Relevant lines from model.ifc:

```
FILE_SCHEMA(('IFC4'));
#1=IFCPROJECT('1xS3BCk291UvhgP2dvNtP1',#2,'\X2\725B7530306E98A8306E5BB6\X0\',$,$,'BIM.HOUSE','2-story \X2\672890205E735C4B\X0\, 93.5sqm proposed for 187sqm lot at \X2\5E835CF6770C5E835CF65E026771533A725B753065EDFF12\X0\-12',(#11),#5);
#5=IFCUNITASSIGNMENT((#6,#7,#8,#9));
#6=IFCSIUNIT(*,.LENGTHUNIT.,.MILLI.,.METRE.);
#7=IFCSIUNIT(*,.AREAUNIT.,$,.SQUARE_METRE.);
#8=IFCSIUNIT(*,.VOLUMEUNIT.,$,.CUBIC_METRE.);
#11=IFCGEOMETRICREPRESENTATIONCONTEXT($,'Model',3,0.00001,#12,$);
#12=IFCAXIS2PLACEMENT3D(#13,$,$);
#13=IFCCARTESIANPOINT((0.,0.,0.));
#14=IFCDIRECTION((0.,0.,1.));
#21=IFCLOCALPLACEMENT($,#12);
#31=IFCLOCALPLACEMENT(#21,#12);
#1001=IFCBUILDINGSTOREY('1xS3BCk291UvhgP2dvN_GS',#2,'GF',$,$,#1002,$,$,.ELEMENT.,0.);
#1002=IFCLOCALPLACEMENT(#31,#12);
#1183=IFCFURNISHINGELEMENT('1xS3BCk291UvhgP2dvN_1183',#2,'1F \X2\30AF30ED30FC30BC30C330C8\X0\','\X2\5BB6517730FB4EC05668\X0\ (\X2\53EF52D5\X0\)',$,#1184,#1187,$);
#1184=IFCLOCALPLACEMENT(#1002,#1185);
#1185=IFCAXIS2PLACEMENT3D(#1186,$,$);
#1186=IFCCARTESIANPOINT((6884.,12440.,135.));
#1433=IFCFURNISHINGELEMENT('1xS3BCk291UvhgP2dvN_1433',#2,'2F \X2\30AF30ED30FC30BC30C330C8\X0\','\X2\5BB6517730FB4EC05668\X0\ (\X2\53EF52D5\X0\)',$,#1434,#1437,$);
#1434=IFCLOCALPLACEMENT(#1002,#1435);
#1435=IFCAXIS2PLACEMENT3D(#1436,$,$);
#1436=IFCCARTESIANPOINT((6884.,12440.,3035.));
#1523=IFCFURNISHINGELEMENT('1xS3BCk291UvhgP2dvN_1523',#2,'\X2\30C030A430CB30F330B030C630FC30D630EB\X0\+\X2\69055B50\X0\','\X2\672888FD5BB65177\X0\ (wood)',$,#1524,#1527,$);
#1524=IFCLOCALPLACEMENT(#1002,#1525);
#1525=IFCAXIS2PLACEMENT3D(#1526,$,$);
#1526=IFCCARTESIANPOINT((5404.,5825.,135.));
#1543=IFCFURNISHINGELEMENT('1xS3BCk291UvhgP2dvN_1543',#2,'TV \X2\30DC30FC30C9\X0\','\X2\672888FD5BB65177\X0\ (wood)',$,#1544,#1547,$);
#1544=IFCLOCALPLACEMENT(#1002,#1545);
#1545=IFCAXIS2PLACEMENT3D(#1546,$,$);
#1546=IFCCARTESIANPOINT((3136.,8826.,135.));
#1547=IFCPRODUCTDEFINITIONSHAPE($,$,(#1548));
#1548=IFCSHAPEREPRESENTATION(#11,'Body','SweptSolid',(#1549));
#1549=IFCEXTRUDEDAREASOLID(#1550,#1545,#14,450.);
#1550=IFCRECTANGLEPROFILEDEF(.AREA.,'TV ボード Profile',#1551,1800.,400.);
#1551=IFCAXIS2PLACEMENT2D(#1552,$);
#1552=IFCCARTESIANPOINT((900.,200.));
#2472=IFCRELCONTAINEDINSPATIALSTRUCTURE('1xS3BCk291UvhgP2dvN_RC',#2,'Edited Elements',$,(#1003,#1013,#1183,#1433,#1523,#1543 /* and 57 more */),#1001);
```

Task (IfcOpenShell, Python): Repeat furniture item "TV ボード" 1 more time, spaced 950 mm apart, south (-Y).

```python
import numpy as np
import ifcopenshell
import ifcopenshell.api.geometry
import ifcopenshell.api.root
import ifcopenshell.util.element
import ifcopenshell.util.placement
import ifcopenshell.util.unit

model = ifcopenshell.open("model.ifc")
unit_scale = ifcopenshell.util.unit.calculate_unit_scale(model)


def reuse_history(source, copy):
    """copy_class also copies each property set's owner history, people and application; keep the originals."""
    for rel in copy.IsDefinedBy:
        if rel.is_a("IfcRelDefinesByProperties") and (history := rel.RelatingPropertyDefinition.OwnerHistory):
            rel.RelatingPropertyDefinition.OwnerHistory = source.OwnerHistory
            ifcopenshell.util.element.remove_deep2(model, history)


source = model.by_id(1543)
base = ifcopenshell.util.placement.get_local_placement(source.ObjectPlacement)
step = np.array([0.0, -1.0, 0.0]) * 0.95 / unit_scale

for i in range(1, 2):
    copy = ifcopenshell.api.root.copy_class(model, product=source)
    copy.Representation = ifcopenshell.util.element.copy_deep(
        model, source.Representation, exclude=["IfcGeometricRepresentationContext", "IfcRepresentationMap"]
    )
    reuse_history(source, copy)
    matrix = base.copy()
    matrix[:3, 3] += i * step
    print("added at", matrix[:3, 3].round(3) + 0.0)
    ifcopenshell.api.geometry.edit_object_placement(model, product=copy, matrix=matrix, is_si=False)

model.write("model_rev.ifc")
```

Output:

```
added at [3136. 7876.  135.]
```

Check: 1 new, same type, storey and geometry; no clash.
